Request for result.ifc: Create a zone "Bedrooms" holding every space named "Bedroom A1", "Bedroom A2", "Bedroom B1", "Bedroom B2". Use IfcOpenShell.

First a look at what the model holds.

```python
import ifcopenshell

model = ifcopenshell.open("result.ifc")
print(model.schema)
seen = {}
for space in model.by_type("IfcSpace"):
    seen[space.Name] = seen.get(space.Name, 0) + 1
for name, count in sorted(seen.items(), key=str):
    print(count, "x", name)
print("zones:", [z.Name for z in model.by_type("IfcZone")][:20])
```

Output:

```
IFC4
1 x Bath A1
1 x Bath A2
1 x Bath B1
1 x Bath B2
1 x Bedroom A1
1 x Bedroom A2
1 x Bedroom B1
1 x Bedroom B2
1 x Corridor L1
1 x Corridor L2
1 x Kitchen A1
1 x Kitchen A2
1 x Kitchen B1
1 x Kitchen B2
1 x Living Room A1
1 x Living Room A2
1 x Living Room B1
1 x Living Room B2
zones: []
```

```python
import ifcopenshell
import ifcopenshell.api.group
import ifcopenshell.api.root

model = ifcopenshell.open("result.ifc")

names = {"Bedroom A1", "Bedroom A2", "Bedroom B1", "Bedroom B2"}
spaces = [s for s in model.by_type("IfcSpace") if s.Name in names]

zone = ifcopenshell.api.root.create_entity(model, ifc_class="IfcZone", name="Bedrooms")
ifcopenshell.api.group.assign_group(model, products=spaces, group=zone)
print(len(spaces), "spaces in", zone.Name)

model.write("result-out.ifc")
```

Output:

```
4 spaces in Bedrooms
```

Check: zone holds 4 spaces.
